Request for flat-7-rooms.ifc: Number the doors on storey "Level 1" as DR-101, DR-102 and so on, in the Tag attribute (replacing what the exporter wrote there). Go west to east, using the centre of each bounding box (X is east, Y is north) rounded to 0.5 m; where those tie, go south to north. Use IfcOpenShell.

First a look at what the model holds.

```python
import ifcopenshell
import ifcopenshell.util.element
import ifcopenshell.util.placement

model = ifcopenshell.open("flat-7-rooms.ifc")
print(model.schema)
storey = next(s for s in model.by_type("IfcBuildingStorey") if s.Name == "Level 1")
doors = [e for e in ifcopenshell.util.element.get_decomposition(storey) if e.is_a("IfcDoor")]
for e in sorted(doors, key=lambda e: e.id()):
    origin = ifcopenshell.util.placement.get_local_placement(e.ObjectPlacement)[:3, 3]
    print(e.id(), e.Tag, e.Name, origin.round(2) + 0.0, sep=" | ")
```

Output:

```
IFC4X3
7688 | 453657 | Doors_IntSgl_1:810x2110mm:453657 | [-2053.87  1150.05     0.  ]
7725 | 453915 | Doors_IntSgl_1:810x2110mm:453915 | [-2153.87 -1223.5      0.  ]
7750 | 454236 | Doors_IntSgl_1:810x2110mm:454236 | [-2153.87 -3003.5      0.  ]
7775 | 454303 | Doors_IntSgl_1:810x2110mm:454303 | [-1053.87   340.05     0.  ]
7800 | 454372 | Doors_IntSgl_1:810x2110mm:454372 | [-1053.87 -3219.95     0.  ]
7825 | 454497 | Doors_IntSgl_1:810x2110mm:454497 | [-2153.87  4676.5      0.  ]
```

```python
import ifcopenshell
import ifcopenshell.geom
import ifcopenshell.util.element
import ifcopenshell.util.shape

model = ifcopenshell.open("flat-7-rooms.ifc")
settings = ifcopenshell.geom.settings()
settings.set("use-world-coords", True)


def centre(element):
    shape = ifcopenshell.geom.create_shape(settings, element)
    return ifcopenshell.util.shape.get_bbox_centroid(shape.geometry)


storey = next(s for s in model.by_type("IfcBuildingStorey") if s.Name == "Level 1")
doors = [e for e in ifcopenshell.util.element.get_decomposition(storey) if e.is_a("IfcDoor")]

# Insertion points can sit at a corner or the storey origin, so sort by the geometry (in metres).
centres = {e: centre(e) for e in doors}
doors.sort(key=lambda e: (round(centres[e][0] / 0.5), centres[e][1]))

for i, e in enumerate(doors, start=1):
    number = f"DR-1{i:02d}"
    e.Tag = number
    print(e.id(), number)

model.write("flat-7-rooms_rev.ifc")
```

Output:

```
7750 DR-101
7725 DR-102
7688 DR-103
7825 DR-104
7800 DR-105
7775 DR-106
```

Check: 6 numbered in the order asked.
